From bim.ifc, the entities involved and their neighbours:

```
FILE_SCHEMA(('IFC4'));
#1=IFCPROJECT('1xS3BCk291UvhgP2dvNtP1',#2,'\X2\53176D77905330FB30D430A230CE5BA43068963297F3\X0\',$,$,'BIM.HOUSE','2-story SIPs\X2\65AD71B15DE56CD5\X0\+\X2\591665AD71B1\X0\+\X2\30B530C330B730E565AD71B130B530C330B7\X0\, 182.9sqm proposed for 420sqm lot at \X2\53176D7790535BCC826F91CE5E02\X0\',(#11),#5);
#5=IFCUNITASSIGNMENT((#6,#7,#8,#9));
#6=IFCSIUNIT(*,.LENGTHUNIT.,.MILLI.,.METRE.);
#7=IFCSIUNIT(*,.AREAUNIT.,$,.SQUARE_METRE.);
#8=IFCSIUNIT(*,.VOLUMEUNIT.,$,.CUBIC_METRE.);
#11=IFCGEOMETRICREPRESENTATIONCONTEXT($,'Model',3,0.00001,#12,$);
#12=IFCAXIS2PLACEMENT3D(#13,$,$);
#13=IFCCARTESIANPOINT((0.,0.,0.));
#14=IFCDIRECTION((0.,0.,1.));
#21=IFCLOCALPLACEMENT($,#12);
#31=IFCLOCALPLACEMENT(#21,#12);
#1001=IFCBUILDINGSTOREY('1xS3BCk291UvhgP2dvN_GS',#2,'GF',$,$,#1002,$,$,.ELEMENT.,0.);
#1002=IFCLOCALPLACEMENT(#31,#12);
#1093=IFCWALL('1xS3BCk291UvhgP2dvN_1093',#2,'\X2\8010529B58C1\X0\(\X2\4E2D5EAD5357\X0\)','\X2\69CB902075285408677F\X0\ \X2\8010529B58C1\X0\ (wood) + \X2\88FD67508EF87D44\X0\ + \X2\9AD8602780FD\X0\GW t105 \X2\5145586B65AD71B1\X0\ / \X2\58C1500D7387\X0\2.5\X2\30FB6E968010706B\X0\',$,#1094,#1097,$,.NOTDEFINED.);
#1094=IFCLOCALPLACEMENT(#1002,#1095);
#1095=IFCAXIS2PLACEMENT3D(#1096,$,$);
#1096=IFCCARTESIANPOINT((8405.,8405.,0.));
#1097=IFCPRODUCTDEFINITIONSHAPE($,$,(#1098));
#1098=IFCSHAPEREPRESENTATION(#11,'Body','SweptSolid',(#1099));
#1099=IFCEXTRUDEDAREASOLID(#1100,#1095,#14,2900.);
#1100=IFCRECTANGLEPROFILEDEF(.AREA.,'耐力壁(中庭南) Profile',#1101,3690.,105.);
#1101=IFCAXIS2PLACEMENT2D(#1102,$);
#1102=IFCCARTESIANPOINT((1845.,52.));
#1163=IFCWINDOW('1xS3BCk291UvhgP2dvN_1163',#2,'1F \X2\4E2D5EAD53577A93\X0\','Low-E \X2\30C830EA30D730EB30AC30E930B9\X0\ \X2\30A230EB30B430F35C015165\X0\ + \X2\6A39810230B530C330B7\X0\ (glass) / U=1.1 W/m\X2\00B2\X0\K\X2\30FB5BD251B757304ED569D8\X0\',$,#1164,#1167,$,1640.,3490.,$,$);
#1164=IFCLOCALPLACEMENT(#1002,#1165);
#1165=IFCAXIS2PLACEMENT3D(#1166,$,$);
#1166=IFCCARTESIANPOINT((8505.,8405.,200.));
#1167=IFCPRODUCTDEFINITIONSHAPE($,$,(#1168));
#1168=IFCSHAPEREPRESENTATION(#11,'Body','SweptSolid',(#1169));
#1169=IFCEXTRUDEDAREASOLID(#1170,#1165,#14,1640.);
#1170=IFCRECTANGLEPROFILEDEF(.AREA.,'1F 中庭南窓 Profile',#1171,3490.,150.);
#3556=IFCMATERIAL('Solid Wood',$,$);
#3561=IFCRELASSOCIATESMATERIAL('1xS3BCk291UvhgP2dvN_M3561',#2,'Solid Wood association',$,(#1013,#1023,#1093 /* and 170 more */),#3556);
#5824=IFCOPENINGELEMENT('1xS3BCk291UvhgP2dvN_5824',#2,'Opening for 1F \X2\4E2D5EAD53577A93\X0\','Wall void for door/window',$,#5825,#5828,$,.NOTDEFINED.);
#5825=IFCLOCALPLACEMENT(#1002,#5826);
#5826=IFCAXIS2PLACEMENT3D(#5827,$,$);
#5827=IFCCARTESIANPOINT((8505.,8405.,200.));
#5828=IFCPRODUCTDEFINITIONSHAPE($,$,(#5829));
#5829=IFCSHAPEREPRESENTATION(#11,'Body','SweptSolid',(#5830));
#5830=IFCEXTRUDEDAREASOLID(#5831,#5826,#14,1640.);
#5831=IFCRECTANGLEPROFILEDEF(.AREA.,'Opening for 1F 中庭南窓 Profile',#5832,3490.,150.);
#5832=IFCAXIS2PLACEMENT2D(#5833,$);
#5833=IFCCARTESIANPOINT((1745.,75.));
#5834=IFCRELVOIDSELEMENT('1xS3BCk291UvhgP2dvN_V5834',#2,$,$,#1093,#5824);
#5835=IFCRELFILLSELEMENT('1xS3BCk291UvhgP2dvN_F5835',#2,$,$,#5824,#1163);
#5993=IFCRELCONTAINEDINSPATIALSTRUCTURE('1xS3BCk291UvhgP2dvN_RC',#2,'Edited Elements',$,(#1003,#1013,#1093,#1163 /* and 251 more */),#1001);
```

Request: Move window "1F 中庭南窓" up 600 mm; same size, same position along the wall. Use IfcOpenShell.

```python
import numpy as np
import ifcopenshell
import ifcopenshell.api.geometry
import ifcopenshell.util.placement
import ifcopenshell.util.unit

model = ifcopenshell.open("bim.ifc")
unit_scale = ifcopenshell.util.unit.calculate_unit_scale(model)

window = model.by_id(1163)
opening = window.FillsVoids[0].RelatingOpeningElement
dz = 0.6 / unit_scale

shift = np.array([0.0, 0.0, dz])
# The window is not placed relative to its opening, so move both.
for product in (opening, window):
    matrix = ifcopenshell.util.placement.get_local_placement(product.ObjectPlacement)
    matrix[:3, 3] += shift
    ifcopenshell.api.geometry.edit_object_placement(model, product=product, matrix=matrix, is_si=False)

print(f"moved by {dz * unit_scale:+.3f} m")

model.write("bim-out.ifc")
```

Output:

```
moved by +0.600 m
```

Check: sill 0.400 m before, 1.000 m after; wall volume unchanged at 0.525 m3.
